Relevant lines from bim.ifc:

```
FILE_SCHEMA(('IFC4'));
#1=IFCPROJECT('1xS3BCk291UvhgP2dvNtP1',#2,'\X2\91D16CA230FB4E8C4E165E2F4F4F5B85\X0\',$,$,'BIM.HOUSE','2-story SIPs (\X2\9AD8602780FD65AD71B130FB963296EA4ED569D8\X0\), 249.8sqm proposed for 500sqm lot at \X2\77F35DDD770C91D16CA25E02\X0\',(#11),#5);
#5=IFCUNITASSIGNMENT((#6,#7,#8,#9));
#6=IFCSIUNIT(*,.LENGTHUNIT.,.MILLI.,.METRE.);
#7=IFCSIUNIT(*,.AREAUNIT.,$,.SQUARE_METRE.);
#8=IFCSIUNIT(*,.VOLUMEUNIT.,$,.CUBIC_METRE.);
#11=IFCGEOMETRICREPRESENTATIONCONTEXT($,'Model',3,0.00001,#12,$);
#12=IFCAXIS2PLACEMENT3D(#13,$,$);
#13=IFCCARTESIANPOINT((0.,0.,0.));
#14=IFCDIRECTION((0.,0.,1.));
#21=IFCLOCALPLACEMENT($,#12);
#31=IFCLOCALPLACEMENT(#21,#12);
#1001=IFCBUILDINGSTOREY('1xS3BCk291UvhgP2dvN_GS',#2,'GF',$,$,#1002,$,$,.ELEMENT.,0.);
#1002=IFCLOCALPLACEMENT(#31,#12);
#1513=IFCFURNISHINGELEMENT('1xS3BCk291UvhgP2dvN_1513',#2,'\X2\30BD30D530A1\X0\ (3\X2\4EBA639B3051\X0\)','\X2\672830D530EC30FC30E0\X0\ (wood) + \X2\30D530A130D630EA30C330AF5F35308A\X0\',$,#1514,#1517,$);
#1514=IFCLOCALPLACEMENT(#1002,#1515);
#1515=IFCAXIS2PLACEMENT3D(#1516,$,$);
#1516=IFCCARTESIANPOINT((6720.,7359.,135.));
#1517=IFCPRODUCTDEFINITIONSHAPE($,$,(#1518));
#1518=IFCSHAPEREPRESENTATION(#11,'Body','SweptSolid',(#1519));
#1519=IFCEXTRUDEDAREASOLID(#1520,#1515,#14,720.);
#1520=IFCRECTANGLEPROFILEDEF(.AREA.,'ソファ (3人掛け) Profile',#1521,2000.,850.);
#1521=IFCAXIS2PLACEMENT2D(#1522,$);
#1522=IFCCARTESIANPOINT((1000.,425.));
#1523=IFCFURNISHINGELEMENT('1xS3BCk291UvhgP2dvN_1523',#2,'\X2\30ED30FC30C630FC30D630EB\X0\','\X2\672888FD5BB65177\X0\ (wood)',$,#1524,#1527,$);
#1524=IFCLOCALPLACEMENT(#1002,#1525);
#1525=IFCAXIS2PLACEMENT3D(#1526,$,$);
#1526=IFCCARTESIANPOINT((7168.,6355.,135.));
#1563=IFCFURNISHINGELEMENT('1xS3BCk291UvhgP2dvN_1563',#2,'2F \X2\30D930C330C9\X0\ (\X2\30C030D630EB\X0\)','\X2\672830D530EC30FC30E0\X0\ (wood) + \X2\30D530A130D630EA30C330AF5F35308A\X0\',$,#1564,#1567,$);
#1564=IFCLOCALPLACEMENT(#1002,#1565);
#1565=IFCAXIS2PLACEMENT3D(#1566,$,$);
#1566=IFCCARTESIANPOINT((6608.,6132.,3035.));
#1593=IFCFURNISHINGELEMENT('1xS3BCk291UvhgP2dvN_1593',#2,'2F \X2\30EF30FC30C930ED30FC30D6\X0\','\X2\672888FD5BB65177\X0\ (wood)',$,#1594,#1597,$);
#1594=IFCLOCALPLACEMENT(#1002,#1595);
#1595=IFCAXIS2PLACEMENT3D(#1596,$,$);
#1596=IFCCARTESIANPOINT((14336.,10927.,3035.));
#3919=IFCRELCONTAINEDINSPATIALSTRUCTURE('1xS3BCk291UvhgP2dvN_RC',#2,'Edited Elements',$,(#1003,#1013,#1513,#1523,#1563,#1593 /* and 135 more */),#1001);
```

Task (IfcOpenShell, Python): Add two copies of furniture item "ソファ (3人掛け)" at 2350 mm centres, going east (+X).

```python
import numpy as np
import ifcopenshell
import ifcopenshell.api.geometry
import ifcopenshell.api.root
import ifcopenshell.util.element
import ifcopenshell.util.placement
import ifcopenshell.util.unit

model = ifcopenshell.open("bim.ifc")
unit_scale = ifcopenshell.util.unit.calculate_unit_scale(model)


def reuse_history(source, copy):
    """copy_class also copies each property set's owner history, people and application; keep the originals."""
    for rel in copy.IsDefinedBy:
        if rel.is_a("IfcRelDefinesByProperties") and (history := rel.RelatingPropertyDefinition.OwnerHistory):
            rel.RelatingPropertyDefinition.OwnerHistory = source.OwnerHistory
            ifcopenshell.util.element.remove_deep2(model, history)


source = model.by_guid("1xS3BCk291UvhgP2dvN_1513")
base = ifcopenshell.util.placement.get_local_placement(source.ObjectPlacement)
step = np.array([1.0, 0.0, 0.0]) * 2.35 / unit_scale

for i in range(1, 3):
    copy = ifcopenshell.api.root.copy_class(model, product=source)
    copy.Representation = ifcopenshell.util.element.copy_deep(
        model, source.Representation, exclude=["IfcGeometricRepresentationContext", "IfcRepresentationMap"]
    )
    reuse_history(source, copy)
    matrix = base.copy()
    matrix[:3, 3] += i * step
    print("added at", matrix[:3, 3].round(3) + 0.0)
    ifcopenshell.api.geometry.edit_object_placement(model, product=copy, matrix=matrix, is_si=False)

model.write("bim_edited.ifc")
```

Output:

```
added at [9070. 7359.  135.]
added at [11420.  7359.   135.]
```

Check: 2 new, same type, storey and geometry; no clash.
